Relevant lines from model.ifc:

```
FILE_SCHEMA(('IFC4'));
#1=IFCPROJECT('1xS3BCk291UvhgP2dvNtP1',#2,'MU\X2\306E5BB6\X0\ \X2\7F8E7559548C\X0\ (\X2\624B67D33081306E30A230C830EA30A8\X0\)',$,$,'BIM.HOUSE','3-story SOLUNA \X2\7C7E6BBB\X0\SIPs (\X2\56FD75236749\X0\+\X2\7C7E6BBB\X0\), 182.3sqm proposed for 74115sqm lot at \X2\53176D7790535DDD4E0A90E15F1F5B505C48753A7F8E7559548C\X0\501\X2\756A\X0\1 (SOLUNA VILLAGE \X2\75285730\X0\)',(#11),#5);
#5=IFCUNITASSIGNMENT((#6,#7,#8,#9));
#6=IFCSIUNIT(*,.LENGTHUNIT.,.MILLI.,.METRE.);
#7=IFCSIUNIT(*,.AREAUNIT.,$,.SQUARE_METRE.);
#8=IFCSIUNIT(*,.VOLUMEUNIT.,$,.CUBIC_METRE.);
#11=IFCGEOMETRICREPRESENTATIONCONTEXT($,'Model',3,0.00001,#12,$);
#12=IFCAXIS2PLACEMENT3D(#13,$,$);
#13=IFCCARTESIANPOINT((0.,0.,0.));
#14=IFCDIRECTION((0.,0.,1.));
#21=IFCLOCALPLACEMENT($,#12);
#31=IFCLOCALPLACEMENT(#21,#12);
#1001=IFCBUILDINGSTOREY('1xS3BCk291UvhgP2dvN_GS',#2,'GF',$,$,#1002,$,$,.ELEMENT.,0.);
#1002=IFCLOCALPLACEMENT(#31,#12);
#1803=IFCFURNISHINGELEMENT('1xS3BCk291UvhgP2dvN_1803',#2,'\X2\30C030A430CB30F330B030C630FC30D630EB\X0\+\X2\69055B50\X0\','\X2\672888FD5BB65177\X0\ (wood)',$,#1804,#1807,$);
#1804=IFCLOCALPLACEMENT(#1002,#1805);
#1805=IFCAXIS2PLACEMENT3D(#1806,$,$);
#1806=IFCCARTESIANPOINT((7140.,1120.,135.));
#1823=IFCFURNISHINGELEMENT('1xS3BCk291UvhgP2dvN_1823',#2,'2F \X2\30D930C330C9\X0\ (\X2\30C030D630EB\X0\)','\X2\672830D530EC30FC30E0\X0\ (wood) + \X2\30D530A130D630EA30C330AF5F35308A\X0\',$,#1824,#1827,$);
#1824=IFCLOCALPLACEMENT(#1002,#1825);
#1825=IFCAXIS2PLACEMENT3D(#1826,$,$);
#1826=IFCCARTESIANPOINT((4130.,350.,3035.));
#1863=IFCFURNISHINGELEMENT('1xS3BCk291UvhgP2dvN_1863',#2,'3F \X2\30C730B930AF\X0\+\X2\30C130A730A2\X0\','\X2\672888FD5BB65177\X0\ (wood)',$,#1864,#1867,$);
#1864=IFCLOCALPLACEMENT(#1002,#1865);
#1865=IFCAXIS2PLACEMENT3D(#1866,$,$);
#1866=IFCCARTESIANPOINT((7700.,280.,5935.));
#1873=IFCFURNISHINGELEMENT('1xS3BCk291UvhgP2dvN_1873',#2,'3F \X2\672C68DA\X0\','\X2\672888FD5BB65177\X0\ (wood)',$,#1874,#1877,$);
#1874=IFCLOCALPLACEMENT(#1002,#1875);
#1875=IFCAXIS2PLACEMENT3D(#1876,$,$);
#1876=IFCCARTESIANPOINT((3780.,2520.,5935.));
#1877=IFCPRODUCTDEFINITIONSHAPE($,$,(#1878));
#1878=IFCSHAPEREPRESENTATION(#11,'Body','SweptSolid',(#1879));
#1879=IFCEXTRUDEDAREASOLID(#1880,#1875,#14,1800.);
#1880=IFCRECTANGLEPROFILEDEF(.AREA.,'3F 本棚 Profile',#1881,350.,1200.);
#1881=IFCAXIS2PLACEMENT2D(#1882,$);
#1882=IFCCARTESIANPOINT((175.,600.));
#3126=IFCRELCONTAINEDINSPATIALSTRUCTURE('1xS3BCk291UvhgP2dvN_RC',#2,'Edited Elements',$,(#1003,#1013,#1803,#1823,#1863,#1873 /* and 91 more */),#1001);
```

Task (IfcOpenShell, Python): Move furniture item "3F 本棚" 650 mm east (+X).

```python
import ifcopenshell
import ifcopenshell.api.geometry
import ifcopenshell.util.placement
import ifcopenshell.util.unit

model = ifcopenshell.open("model.ifc")
unit_scale = ifcopenshell.util.unit.calculate_unit_scale(model)

item = model.by_guid("1xS3BCk291UvhgP2dvN_1873")
matrix = ifcopenshell.util.placement.get_local_placement(item.ObjectPlacement)
matrix[0, 3] += 0.65 / unit_scale
ifcopenshell.api.geometry.edit_object_placement(model, product=item, matrix=matrix, is_si=False)

print(ifcopenshell.util.placement.get_local_placement(item.ObjectPlacement).round(3) + 0.0)

model.write("model_v2.ifc")
```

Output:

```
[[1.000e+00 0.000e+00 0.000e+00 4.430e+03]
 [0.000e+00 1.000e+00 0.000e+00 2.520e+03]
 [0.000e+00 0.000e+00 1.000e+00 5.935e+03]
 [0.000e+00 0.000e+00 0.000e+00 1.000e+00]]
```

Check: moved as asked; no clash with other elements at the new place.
